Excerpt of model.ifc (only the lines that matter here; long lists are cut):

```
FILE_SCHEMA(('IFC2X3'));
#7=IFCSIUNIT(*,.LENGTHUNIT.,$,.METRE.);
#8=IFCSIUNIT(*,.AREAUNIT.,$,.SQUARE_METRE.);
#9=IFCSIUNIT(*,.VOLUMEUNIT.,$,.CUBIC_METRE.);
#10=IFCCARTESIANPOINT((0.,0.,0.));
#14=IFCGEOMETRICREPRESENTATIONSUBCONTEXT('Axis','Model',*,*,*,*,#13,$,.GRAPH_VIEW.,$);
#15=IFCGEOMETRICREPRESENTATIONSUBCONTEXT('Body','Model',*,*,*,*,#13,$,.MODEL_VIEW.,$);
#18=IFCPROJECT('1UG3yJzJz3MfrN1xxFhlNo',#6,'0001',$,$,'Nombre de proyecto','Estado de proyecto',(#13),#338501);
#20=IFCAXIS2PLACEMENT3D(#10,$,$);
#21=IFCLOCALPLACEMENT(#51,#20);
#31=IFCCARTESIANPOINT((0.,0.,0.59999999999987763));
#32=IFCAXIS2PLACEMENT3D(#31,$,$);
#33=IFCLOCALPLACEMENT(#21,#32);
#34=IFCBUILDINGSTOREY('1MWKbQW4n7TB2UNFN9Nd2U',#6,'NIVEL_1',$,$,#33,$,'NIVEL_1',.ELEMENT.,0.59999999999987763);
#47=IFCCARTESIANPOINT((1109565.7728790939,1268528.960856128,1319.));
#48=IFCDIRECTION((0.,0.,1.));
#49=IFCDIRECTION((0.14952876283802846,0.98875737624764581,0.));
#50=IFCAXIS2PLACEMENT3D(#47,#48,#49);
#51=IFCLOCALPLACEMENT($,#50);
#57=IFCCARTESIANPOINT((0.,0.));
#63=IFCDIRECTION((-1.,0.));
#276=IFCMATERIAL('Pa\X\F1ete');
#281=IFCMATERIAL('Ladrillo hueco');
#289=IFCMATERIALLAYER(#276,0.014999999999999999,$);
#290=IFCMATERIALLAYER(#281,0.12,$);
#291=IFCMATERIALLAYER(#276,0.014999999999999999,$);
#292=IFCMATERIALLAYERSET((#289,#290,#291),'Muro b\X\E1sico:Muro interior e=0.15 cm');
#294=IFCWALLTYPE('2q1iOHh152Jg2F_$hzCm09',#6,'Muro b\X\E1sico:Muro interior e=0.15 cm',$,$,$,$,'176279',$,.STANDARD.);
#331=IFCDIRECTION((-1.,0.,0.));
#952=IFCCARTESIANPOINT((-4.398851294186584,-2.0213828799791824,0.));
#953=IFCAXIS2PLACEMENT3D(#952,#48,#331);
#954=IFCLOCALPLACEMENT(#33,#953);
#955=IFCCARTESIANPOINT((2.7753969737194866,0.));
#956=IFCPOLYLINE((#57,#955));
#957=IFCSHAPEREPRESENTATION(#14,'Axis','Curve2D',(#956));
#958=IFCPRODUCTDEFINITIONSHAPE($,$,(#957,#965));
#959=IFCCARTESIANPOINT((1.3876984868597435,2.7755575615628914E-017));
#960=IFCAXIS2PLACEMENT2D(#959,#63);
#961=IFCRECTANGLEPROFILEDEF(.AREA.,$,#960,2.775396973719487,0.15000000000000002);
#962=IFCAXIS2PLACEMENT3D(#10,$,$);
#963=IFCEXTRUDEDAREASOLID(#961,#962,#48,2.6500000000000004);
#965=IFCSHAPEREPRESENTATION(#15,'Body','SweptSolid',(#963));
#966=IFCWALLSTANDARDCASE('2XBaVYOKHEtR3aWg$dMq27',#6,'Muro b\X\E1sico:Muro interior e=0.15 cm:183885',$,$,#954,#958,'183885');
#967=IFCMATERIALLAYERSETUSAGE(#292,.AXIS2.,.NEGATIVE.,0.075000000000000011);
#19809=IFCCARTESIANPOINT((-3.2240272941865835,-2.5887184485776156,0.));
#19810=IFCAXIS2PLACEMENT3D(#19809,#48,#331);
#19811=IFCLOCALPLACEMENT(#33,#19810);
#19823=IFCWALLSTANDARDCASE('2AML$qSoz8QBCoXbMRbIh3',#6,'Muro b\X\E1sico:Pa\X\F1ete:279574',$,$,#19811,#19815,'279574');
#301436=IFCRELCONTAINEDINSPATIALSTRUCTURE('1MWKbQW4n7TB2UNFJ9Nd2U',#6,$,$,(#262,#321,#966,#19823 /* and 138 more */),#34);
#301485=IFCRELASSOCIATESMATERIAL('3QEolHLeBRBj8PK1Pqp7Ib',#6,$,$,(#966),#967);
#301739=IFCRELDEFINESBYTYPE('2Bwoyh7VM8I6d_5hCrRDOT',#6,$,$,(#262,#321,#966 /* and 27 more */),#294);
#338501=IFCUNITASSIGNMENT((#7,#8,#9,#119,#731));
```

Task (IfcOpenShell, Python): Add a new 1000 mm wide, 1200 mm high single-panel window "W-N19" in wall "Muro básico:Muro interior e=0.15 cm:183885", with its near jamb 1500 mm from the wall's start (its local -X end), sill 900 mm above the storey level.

```python
import numpy as np
import ifcopenshell
import ifcopenshell.api.feature
import ifcopenshell.api.geometry
import ifcopenshell.api.root
import ifcopenshell.api.spatial
import ifcopenshell.api.type
import ifcopenshell.geom
import ifcopenshell.util.element
import ifcopenshell.util.placement
import ifcopenshell.util.representation
import ifcopenshell.util.shape
import ifcopenshell.util.unit

model = ifcopenshell.open("model.ifc")
unit_scale = ifcopenshell.util.unit.calculate_unit_scale(model)
settings = ifcopenshell.geom.settings()


def volume(element):
    """Net volume in cubic metres, openings subtracted."""
    shape = ifcopenshell.geom.create_shape(settings, element)
    return ifcopenshell.util.shape.get_volume(shape.geometry)


wall = model.by_guid("2XBaVYOKHEtR3aWg$dMq27")
storey = ifcopenshell.util.element.get_container(wall, ifc_class="IfcBuildingStorey")
context = ifcopenshell.util.representation.get_context(model, "Model", "Body", "MODEL_VIEW")
before = volume(wall)

width, height, from_end, sill = 1, 1.2, 1.5, 0.9  # metres

# The wall runs along its own X axis, and the end named is its -X end.
wall_shape = ifcopenshell.geom.create_shape(settings, wall)
x, y, z = ifcopenshell.util.shape.get_vertices(wall_shape.geometry).T
start = x.min() + from_end
face, thickness = float(y.min()), float(y.max() - y.min())
wall_matrix = ifcopenshell.util.placement.get_local_placement(wall.ObjectPlacement)
level = ifcopenshell.util.placement.get_local_placement(storey.ObjectPlacement)[2, 3]


def in_wall(x, y):
    """Placement at x, y metres in the wall's axes, at sill height."""
    matrix = wall_matrix.copy()
    matrix[:, 3] = wall_matrix @ np.array([x / unit_scale, y / unit_scale, 0.0, 1.0])
    matrix[2, 3] = level + sill / unit_scale
    return matrix


# Opening: a box that overshoots both wall faces by 50 mm.
opening = ifcopenshell.api.root.create_entity(model, ifc_class="IfcOpeningElement")
box = ifcopenshell.api.geometry.add_wall_representation(
    model, context=context, length=width, height=height, thickness=thickness + 0.1
)
ifcopenshell.api.geometry.assign_representation(model, product=opening, representation=box)
ifcopenshell.api.geometry.edit_object_placement(model, product=opening, matrix=in_wall(start, face - 0.05), is_si=False)
ifcopenshell.api.feature.add_feature(model, feature=opening, element=wall)

window = ifcopenshell.api.root.create_entity(model, ifc_class="IfcWindow", name="W-N19")
window.OverallWidth, window.OverallHeight = width / unit_scale, height / unit_scale
body = ifcopenshell.api.geometry.add_window_representation(
    model,
    context=context,
    overall_width=window.OverallWidth,
    overall_height=window.OverallHeight,
    partition_type="SINGLE_PANEL",
)
ifcopenshell.api.geometry.assign_representation(model, product=window, representation=body)
ifcopenshell.api.spatial.assign_container(model, products=[window], relating_structure=storey)
fills = ifcopenshell.api.feature.add_filling(model, opening=opening, element=window)
fills.OwnerHistory = window.OwnerHistory  # required in IFC2X3

# IFC2X3 keeps the operation on the window style.
style = ifcopenshell.api.root.create_entity(model, ifc_class="IfcWindowStyle", name="W-N19")
style.OperationType, style.ConstructionType = "SINGLE_PANEL", "NOTDEFINED"
style.ParameterTakesPrecedence = style.Sizeable = False
ifcopenshell.api.type.assign_type(model, related_objects=[window], relating_type=style)

# Centre the window in the wall's thickness.
ifcopenshell.api.geometry.edit_object_placement(model, product=window, matrix=in_wall(start, face), is_si=False)
window_shape = ifcopenshell.geom.create_shape(settings, window)
depth = ifcopenshell.util.shape.get_vertices(window_shape.geometry)[:, 1]
offset = face + thickness / 2 - (depth.min() + depth.max()) / 2
ifcopenshell.api.geometry.edit_object_placement(model, product=window, matrix=in_wall(start, offset), is_si=False)

after = volume(wall)

print(f"wall volume {before:.3f} -> {after:.3f} m3")

model.write("model_rev.ifc")
```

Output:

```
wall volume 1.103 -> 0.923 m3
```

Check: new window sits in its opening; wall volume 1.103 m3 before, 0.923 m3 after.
